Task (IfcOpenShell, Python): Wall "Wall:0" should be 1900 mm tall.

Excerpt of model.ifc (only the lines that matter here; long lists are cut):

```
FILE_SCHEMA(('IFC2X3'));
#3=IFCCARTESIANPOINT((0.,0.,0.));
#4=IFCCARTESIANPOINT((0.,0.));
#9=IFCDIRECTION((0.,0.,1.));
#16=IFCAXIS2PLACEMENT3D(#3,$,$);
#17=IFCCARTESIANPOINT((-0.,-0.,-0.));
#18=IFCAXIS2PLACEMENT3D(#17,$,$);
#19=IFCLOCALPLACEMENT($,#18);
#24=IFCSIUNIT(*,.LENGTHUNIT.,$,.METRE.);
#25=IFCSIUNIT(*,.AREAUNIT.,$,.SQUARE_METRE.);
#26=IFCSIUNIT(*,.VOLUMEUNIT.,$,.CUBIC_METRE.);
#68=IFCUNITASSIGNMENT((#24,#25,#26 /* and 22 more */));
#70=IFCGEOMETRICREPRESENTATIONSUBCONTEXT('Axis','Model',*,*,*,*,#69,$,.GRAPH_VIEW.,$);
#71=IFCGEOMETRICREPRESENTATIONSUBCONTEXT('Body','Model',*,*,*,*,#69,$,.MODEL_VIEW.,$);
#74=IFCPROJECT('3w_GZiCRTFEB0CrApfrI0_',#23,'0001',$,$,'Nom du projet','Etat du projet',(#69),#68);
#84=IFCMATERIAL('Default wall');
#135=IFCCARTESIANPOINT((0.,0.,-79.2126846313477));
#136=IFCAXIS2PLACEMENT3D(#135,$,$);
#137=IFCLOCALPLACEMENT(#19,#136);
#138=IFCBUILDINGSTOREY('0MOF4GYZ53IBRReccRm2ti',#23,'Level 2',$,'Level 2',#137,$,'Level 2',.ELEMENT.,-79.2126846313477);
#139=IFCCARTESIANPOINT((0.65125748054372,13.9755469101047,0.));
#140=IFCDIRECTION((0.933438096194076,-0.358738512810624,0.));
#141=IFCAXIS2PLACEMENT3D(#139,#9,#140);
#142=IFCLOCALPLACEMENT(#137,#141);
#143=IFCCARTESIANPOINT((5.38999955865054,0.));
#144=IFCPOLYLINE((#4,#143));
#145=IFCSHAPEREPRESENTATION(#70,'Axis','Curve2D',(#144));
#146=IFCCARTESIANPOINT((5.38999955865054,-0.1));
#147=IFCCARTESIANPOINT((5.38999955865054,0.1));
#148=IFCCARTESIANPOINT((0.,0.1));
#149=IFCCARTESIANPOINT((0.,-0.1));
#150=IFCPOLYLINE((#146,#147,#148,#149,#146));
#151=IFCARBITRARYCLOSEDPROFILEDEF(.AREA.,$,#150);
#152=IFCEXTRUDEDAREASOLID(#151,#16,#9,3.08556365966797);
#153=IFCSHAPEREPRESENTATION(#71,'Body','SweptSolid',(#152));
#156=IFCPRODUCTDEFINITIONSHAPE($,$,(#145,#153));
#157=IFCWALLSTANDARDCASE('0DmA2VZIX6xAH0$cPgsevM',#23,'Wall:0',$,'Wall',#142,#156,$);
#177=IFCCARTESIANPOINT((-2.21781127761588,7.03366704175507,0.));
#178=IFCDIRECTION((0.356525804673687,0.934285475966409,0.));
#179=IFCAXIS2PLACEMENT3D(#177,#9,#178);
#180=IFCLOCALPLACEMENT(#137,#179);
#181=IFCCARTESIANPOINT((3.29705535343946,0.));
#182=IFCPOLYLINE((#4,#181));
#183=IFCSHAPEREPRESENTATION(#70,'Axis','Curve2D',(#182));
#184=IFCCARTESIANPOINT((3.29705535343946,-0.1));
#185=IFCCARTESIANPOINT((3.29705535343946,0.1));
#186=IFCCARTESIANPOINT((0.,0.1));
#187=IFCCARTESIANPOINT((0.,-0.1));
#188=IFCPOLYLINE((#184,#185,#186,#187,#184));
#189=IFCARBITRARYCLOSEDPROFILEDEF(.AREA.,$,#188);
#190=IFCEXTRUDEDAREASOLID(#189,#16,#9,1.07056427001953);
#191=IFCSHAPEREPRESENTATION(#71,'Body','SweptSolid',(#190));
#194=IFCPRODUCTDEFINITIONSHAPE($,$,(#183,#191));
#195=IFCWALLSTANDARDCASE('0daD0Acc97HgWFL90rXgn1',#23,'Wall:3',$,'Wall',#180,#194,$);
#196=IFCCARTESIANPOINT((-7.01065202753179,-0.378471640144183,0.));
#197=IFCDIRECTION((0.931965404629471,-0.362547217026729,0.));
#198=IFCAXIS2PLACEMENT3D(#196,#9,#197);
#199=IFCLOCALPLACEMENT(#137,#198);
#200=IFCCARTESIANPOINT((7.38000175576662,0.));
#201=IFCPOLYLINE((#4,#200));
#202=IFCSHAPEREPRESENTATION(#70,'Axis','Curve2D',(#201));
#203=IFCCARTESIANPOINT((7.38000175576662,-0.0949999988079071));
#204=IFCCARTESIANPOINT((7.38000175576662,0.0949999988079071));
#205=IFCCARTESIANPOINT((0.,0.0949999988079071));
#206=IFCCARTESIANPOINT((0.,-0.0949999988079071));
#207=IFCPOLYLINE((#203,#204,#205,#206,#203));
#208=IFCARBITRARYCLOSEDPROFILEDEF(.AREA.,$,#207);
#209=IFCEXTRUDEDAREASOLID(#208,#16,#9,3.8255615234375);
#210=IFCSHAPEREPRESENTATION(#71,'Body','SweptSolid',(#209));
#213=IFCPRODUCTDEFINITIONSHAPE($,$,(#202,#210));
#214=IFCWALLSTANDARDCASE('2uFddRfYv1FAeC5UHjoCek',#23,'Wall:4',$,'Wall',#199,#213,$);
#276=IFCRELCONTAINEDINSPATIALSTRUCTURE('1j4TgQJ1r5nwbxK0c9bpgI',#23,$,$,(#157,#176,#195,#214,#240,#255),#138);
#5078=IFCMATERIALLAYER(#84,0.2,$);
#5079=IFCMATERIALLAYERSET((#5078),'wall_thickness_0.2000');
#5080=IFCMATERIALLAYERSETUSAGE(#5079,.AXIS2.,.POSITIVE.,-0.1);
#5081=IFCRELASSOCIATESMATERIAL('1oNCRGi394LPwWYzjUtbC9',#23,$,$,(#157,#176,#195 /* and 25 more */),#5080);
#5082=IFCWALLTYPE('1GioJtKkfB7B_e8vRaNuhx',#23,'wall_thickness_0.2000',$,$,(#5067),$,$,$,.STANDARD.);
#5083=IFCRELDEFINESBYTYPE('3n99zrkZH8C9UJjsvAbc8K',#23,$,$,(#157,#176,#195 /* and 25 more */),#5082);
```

```python
import ifcopenshell
import ifcopenshell.geom
import ifcopenshell.util.representation
import ifcopenshell.util.shape

model = ifcopenshell.open("model.ifc")
settings = ifcopenshell.geom.settings()


def volume(element):
    """Net volume in cubic metres, openings subtracted."""
    shape = ifcopenshell.geom.create_shape(settings, element)
    return ifcopenshell.util.shape.get_volume(shape.geometry)


wall = model.by_id(157)
before = volume(wall)

body = ifcopenshell.util.representation.get_representation(wall, "Model", "Body")
solid = body.Items[0]
old_height = solid.Depth
solid.Depth = 1.9
after = volume(wall)

print(f"height {old_height:g} -> {solid.Depth:g}, volume {before:.3f} -> {after:.3f} m3")

model.write("model_rev.ifc")
```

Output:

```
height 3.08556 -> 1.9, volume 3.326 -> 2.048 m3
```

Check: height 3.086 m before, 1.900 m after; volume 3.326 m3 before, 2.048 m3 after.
